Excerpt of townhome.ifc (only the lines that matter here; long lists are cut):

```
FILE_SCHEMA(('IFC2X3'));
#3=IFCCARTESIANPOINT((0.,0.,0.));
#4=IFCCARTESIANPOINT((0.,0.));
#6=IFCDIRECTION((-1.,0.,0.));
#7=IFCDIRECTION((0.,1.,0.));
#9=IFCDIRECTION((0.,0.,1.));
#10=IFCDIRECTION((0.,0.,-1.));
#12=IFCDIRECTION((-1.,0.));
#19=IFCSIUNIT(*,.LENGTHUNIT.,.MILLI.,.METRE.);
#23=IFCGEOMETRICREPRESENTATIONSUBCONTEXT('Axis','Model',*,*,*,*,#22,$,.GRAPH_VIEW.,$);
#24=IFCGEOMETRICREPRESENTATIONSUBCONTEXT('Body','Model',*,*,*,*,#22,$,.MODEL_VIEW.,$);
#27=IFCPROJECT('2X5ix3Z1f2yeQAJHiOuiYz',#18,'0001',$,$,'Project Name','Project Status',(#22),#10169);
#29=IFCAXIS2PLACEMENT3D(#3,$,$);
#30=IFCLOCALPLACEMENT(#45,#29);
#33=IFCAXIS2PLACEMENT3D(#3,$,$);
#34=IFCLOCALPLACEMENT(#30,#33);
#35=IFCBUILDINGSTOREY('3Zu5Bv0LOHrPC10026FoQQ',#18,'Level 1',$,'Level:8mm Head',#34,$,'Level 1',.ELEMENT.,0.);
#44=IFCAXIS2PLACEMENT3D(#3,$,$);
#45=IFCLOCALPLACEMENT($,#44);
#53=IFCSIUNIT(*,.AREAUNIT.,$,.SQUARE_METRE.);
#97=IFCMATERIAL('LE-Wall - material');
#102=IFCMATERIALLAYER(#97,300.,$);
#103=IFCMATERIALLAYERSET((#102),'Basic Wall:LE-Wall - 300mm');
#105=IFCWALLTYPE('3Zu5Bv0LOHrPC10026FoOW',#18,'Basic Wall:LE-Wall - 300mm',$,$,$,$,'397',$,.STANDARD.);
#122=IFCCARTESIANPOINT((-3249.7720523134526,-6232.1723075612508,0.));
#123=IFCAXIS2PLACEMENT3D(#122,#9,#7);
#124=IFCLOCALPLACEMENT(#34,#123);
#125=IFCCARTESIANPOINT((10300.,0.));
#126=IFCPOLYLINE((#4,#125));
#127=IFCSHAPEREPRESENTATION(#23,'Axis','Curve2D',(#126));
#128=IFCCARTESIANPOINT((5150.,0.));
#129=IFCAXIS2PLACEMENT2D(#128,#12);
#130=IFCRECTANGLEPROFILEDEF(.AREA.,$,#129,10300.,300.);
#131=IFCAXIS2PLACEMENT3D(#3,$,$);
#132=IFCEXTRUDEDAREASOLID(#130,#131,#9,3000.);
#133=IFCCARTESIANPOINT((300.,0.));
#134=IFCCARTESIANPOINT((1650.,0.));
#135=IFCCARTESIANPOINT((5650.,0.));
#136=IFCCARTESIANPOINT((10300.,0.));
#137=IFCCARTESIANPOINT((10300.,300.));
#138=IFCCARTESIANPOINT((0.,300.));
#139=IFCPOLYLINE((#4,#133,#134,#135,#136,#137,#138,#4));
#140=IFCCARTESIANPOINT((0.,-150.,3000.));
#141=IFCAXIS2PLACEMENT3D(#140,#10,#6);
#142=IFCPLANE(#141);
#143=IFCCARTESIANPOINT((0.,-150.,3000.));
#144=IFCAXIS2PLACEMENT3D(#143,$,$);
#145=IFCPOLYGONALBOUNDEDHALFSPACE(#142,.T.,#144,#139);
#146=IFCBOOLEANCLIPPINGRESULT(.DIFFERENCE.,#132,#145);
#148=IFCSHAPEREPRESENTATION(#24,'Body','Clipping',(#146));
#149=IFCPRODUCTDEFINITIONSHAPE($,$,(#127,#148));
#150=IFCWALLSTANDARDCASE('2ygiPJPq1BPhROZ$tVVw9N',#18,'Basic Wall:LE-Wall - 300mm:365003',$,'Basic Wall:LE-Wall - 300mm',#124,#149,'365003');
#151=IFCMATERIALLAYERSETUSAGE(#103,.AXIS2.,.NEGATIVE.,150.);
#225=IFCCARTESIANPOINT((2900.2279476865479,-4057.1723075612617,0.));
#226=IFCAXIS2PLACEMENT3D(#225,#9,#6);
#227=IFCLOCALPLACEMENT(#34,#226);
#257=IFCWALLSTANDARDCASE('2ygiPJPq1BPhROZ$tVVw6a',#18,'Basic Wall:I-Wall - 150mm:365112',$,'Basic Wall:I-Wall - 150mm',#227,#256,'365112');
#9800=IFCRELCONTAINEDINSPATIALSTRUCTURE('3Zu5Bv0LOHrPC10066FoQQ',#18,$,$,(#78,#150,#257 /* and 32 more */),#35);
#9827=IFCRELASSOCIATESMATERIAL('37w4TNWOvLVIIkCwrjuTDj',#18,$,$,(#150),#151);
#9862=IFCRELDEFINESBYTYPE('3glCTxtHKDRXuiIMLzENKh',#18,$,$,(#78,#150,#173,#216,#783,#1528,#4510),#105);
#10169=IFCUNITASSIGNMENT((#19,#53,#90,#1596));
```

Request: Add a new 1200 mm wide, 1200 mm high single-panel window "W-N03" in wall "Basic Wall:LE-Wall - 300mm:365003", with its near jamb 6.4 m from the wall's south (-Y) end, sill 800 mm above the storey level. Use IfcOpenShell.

```python
import numpy as np
import ifcopenshell
import ifcopenshell.api.feature
import ifcopenshell.api.geometry
import ifcopenshell.api.root
import ifcopenshell.api.spatial
import ifcopenshell.api.type
import ifcopenshell.geom
import ifcopenshell.util.element
import ifcopenshell.util.placement
import ifcopenshell.util.representation
import ifcopenshell.util.shape
import ifcopenshell.util.unit

model = ifcopenshell.open("townhome.ifc")
unit_scale = ifcopenshell.util.unit.calculate_unit_scale(model)
settings = ifcopenshell.geom.settings()


def volume(element):
    """Net volume in cubic metres, openings subtracted."""
    shape = ifcopenshell.geom.create_shape(settings, element)
    return ifcopenshell.util.shape.get_volume(shape.geometry)


wall = model.by_guid("2ygiPJPq1BPhROZ$tVVw9N")
storey = ifcopenshell.util.element.get_container(wall, ifc_class="IfcBuildingStorey")
context = ifcopenshell.util.representation.get_context(model, "Model", "Body", "MODEL_VIEW")
before = volume(wall)

width, height, from_end, sill = 1.2, 1.2, 6.4, 0.8  # metres

# The wall runs along its own X axis, and the end named is its -X end.
wall_shape = ifcopenshell.geom.create_shape(settings, wall)
x, y, z = ifcopenshell.util.shape.get_vertices(wall_shape.geometry).T
start = x.min() + from_end
face, thickness = float(y.min()), float(y.max() - y.min())
wall_matrix = ifcopenshell.util.placement.get_local_placement(wall.ObjectPlacement)
level = ifcopenshell.util.placement.get_local_placement(storey.ObjectPlacement)[2, 3]


def in_wall(x, y):
    """Placement at x, y metres in the wall's axes, at sill height."""
    matrix = wall_matrix.copy()
    matrix[:, 3] = wall_matrix @ np.array([x / unit_scale, y / unit_scale, 0.0, 1.0])
    matrix[2, 3] = level + sill / unit_scale
    return matrix


# Opening: a box that overshoots both wall faces by 50 mm.
opening = ifcopenshell.api.root.create_entity(model, ifc_class="IfcOpeningElement")
box = ifcopenshell.api.geometry.add_wall_representation(
    model, context=context, length=width, height=height, thickness=thickness + 0.1
)
ifcopenshell.api.geometry.assign_representation(model, product=opening, representation=box)
ifcopenshell.api.geometry.edit_object_placement(model, product=opening, matrix=in_wall(start, face - 0.05), is_si=False)
ifcopenshell.api.feature.add_feature(model, feature=opening, element=wall)

window = ifcopenshell.api.root.create_entity(model, ifc_class="IfcWindow", name="W-N03")
window.OverallWidth, window.OverallHeight = width / unit_scale, height / unit_scale
body = ifcopenshell.api.geometry.add_window_representation(
    model,
    context=context,
    overall_width=window.OverallWidth,
    overall_height=window.OverallHeight,
    partition_type="SINGLE_PANEL",
)
ifcopenshell.api.geometry.assign_representation(model, product=window, representation=body)
ifcopenshell.api.spatial.assign_container(model, products=[window], relating_structure=storey)
fills = ifcopenshell.api.feature.add_filling(model, opening=opening, element=window)
fills.OwnerHistory = window.OwnerHistory  # required in IFC2X3

# IFC2X3 keeps the operation on the window style.
style = ifcopenshell.api.root.create_entity(model, ifc_class="IfcWindowStyle", name="W-N03")
style.OperationType, style.ConstructionType = "SINGLE_PANEL", "NOTDEFINED"
style.ParameterTakesPrecedence = style.Sizeable = False
ifcopenshell.api.type.assign_type(model, related_objects=[window], relating_type=style)

# Centre the window in the wall's thickness.
ifcopenshell.api.geometry.edit_object_placement(model, product=window, matrix=in_wall(start, face), is_si=False)
window_shape = ifcopenshell.geom.create_shape(settings, window)
depth = ifcopenshell.util.shape.get_vertices(window_shape.geometry)[:, 1]
offset = face + thickness / 2 - (depth.min() + depth.max()) / 2
ifcopenshell.api.geometry.edit_object_placement(model, product=window, matrix=in_wall(start, offset), is_si=False)

after = volume(wall)

print(f"wall volume {before:.3f} -> {after:.3f} m3")

model.write("townhome_edited.ifc")
```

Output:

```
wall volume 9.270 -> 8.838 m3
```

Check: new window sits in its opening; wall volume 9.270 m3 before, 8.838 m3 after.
